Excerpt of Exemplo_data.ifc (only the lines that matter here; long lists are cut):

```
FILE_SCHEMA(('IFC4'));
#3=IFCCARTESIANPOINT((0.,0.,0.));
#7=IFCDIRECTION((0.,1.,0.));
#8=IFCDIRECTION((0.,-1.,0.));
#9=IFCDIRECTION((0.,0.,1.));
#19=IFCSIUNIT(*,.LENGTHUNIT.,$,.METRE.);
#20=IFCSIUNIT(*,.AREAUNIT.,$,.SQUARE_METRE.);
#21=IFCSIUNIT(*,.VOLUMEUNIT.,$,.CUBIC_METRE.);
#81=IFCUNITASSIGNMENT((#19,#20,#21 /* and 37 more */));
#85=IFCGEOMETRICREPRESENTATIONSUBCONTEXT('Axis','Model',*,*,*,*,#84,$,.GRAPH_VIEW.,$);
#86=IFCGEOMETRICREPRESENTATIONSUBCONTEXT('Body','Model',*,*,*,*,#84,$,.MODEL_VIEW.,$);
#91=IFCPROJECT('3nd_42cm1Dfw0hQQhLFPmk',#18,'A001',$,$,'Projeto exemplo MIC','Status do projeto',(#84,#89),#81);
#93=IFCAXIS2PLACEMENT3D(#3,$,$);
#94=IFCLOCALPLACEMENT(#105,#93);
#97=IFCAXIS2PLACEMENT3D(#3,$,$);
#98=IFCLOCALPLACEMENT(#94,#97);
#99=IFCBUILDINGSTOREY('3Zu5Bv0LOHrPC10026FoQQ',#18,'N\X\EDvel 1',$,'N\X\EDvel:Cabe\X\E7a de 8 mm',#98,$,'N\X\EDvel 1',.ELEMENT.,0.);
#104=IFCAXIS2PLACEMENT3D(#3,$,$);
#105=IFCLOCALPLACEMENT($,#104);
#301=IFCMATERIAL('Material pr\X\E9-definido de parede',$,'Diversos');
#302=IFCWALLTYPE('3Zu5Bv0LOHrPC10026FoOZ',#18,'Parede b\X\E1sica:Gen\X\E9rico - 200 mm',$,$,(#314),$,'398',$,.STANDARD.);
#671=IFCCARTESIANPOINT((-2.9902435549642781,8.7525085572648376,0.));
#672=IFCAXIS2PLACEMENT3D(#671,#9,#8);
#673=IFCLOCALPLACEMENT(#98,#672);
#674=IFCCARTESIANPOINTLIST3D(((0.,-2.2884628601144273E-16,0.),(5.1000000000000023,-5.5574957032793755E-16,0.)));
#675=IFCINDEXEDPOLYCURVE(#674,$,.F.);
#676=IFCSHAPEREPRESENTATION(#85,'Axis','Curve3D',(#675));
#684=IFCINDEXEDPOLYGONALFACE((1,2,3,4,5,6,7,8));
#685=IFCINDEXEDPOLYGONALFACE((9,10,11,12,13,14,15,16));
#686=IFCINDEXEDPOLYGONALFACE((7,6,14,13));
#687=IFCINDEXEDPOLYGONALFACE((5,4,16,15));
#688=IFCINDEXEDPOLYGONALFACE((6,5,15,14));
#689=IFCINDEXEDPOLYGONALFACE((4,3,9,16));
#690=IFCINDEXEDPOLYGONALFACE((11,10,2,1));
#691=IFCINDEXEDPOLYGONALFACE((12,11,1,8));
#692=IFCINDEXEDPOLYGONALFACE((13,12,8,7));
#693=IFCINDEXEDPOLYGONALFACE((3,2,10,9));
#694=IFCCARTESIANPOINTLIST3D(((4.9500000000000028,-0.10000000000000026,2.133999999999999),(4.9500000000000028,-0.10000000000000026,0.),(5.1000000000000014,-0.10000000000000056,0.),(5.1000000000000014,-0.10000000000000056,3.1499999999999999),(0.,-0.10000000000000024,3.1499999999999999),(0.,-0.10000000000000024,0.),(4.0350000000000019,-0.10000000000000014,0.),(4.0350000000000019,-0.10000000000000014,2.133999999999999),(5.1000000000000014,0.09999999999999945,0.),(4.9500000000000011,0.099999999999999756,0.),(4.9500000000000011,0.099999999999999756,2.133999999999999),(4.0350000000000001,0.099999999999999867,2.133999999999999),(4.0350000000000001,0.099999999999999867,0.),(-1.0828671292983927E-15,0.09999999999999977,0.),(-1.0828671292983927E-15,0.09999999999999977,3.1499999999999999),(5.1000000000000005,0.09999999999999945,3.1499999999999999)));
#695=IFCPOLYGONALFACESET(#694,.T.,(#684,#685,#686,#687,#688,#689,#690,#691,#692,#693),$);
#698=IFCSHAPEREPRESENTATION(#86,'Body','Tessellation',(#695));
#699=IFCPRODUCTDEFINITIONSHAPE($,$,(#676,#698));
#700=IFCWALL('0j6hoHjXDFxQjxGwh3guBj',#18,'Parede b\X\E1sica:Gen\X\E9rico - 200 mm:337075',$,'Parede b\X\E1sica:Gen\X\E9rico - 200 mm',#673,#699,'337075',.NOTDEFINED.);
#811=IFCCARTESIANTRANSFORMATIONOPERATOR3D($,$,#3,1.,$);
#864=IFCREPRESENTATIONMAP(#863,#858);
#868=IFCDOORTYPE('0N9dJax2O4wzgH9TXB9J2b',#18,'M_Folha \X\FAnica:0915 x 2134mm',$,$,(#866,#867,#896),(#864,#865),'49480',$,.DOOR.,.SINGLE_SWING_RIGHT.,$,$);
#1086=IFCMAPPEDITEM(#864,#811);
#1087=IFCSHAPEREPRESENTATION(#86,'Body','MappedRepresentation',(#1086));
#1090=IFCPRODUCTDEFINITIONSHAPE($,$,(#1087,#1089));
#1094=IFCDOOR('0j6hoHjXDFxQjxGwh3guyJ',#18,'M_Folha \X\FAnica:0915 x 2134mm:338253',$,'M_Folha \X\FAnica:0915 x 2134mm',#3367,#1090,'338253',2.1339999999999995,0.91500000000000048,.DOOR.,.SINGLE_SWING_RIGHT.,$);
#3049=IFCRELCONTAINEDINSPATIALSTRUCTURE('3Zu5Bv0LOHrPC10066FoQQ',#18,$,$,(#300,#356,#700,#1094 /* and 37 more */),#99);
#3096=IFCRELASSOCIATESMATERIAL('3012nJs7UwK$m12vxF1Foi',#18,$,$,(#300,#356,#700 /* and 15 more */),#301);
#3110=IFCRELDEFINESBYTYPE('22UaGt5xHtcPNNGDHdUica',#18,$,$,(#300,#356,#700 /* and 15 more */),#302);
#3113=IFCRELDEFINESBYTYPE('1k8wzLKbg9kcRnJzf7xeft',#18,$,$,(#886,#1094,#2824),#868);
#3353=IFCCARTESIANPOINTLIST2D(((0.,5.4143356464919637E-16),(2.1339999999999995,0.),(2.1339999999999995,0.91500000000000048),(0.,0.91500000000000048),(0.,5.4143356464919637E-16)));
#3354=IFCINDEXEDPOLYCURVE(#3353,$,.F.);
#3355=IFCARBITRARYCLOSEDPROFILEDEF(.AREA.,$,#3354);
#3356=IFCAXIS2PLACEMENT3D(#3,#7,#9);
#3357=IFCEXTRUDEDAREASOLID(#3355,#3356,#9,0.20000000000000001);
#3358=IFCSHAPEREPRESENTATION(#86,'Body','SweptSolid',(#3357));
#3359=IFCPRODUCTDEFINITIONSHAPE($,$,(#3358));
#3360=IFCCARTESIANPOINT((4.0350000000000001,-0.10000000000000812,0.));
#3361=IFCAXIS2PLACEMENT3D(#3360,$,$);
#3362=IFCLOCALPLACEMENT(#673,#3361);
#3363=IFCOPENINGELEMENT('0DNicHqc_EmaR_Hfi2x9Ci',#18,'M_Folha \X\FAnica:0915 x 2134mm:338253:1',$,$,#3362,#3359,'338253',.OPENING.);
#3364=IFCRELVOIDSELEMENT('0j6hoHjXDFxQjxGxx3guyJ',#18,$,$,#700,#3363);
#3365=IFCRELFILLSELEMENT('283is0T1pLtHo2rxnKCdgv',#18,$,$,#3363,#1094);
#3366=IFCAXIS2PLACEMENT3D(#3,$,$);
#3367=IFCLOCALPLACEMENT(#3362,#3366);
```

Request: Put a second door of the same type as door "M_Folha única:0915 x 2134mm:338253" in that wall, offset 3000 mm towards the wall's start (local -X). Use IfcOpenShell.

```python
import ifcopenshell
import ifcopenshell.api.feature
import ifcopenshell.api.geometry
import ifcopenshell.api.root
import ifcopenshell.geom
import ifcopenshell.util.element
import ifcopenshell.util.placement
import ifcopenshell.util.shape
import ifcopenshell.util.unit

model = ifcopenshell.open("Exemplo_data.ifc")
unit_scale = ifcopenshell.util.unit.calculate_unit_scale(model)
settings = ifcopenshell.geom.settings()


def volume(element):
    """Net volume in cubic metres, openings subtracted."""
    shape = ifcopenshell.geom.create_shape(settings, element)
    return ifcopenshell.util.shape.get_volume(shape.geometry)


def reuse_history(source, copy):
    """copy_class also copies each property set's owner history, people and application; keep the originals."""
    for rel in copy.IsDefinedBy:
        if rel.is_a("IfcRelDefinesByProperties") and (history := rel.RelatingPropertyDefinition.OwnerHistory):
            rel.RelatingPropertyDefinition.OwnerHistory = source.OwnerHistory
            ifcopenshell.util.element.remove_deep2(model, history)


door = model.by_id(1094)
opening = door.FillsVoids[0].RelatingOpeningElement
wall = opening.VoidsElements[0].RelatingBuildingElement
before = volume(wall)
shift = ifcopenshell.util.placement.get_local_placement(wall.ObjectPlacement)[:3, 0] * -3 / unit_scale

# copy_class copies the void relationship, type, container and properties, but no geometry.
new_opening = ifcopenshell.api.root.copy_class(model, product=opening)
new_opening.Representation = ifcopenshell.util.element.copy_deep(
    model, opening.Representation, exclude=["IfcGeometricRepresentationContext", "IfcRepresentationMap"]
)
new_opening.Name = "M_Folha única:0915 x 2134mm"
new_opening.Tag = None
new_door = ifcopenshell.api.root.copy_class(model, product=door)
new_door.Representation = ifcopenshell.util.element.copy_deep(
    model, door.Representation, exclude=["IfcGeometricRepresentationContext", "IfcRepresentationMap"]
)
new_door.Name = "M_Folha única:0915 x 2134mm"
new_door.Tag = None
reuse_history(door, new_door)
ifcopenshell.api.feature.add_filling(model, opening=new_opening, element=new_door)

for old, new in ((opening, new_opening), (door, new_door)):
    matrix = ifcopenshell.util.placement.get_local_placement(old.ObjectPlacement)
    matrix[:3, 3] += shift
    ifcopenshell.api.geometry.edit_object_placement(model, product=new, matrix=matrix, is_si=False)

after = volume(wall)

print(f"wall volume {before:.3f} -> {after:.3f} m3")

model.write("Exemplo_data_rev.ifc")
```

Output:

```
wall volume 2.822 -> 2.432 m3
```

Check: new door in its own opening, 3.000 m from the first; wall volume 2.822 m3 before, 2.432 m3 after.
